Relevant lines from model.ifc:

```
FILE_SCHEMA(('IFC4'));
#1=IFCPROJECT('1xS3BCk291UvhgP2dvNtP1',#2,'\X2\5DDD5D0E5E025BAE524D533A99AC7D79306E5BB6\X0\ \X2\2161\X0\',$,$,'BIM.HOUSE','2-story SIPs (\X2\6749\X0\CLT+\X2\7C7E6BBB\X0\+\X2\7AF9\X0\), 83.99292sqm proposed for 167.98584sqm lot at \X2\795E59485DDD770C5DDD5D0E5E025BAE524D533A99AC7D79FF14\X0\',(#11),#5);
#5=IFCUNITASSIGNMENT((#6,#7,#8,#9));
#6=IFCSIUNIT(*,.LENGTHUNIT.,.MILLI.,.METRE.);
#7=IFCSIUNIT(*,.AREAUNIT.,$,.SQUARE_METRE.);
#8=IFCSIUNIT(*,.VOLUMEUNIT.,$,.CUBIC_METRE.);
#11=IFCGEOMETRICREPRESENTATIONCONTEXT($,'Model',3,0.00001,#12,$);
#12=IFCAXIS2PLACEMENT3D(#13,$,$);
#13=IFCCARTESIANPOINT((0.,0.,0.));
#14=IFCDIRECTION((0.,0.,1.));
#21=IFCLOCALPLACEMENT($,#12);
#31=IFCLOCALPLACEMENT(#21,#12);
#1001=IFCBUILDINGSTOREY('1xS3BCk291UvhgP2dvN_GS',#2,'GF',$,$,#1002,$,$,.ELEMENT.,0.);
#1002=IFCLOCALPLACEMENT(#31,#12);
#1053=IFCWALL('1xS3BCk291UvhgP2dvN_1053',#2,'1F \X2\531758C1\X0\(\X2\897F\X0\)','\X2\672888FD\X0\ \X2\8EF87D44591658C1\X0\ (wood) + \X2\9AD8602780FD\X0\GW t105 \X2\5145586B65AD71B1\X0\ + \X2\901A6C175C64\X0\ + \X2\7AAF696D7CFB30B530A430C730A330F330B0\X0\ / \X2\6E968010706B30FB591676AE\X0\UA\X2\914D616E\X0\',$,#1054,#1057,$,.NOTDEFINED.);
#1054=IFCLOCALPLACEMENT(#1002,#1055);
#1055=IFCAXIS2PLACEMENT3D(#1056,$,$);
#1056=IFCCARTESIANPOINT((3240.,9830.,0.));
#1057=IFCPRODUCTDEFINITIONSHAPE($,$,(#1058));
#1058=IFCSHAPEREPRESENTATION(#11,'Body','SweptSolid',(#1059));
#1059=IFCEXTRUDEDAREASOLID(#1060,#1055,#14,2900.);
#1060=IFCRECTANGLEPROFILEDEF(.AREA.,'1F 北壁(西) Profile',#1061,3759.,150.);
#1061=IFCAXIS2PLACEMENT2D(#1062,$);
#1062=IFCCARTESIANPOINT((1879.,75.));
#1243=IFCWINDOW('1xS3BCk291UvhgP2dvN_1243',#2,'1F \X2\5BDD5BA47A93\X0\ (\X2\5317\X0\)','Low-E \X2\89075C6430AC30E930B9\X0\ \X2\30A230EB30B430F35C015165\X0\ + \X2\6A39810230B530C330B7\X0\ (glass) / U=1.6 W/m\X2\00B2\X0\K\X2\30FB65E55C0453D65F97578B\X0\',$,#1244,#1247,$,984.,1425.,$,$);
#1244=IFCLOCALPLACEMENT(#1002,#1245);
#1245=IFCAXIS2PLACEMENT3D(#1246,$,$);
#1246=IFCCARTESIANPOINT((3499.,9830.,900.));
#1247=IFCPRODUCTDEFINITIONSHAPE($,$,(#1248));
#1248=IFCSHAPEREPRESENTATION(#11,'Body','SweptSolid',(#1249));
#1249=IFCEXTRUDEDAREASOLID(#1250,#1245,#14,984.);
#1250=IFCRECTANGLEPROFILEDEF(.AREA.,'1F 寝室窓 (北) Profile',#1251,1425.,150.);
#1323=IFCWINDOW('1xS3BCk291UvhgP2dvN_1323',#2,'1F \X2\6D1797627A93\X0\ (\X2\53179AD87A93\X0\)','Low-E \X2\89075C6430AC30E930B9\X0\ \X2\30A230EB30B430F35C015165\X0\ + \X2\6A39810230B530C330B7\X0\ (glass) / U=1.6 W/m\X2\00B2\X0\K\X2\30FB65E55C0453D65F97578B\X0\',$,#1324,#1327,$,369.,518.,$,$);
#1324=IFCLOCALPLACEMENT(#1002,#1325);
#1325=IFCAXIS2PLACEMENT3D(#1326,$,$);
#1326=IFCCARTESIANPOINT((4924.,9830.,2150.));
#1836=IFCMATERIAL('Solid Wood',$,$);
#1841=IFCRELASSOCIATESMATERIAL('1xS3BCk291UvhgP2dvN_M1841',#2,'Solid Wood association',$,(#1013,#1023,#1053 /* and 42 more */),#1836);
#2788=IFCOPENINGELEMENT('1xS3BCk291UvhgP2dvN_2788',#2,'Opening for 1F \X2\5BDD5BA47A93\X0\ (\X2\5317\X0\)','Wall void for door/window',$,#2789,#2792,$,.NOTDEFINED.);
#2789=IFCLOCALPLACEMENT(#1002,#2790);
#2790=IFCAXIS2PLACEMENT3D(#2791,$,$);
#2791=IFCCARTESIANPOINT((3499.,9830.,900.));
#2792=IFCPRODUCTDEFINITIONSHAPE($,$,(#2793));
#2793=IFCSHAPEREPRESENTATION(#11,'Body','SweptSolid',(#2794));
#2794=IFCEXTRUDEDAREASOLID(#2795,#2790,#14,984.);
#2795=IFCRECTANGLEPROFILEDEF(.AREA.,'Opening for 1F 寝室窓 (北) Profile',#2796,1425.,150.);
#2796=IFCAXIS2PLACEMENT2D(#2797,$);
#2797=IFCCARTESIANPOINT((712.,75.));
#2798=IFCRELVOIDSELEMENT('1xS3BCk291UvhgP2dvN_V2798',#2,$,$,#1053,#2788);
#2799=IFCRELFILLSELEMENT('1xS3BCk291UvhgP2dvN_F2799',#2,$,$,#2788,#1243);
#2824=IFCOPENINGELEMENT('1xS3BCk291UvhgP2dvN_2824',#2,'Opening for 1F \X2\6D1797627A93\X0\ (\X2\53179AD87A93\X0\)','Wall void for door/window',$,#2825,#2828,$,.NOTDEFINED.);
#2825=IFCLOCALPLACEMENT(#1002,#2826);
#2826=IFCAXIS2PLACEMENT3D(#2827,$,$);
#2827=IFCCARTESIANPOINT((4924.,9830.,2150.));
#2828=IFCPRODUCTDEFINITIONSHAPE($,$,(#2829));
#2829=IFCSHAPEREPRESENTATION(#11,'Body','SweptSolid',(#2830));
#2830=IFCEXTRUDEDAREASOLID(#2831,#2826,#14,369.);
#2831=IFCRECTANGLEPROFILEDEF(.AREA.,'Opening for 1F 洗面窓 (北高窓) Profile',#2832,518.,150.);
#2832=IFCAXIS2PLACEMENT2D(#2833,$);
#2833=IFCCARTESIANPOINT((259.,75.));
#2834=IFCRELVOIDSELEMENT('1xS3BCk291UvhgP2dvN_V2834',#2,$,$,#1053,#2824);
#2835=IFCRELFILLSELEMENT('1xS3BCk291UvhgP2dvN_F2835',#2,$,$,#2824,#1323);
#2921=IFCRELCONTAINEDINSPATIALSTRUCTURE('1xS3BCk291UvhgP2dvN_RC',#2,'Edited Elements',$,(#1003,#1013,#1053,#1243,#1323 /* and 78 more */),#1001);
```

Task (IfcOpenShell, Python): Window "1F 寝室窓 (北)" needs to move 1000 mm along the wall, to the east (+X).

```python
import ifcopenshell
import ifcopenshell.api.geometry
import ifcopenshell.util.placement
import ifcopenshell.util.unit

model = ifcopenshell.open("model.ifc")
unit_scale = ifcopenshell.util.unit.calculate_unit_scale(model)

window = model.by_guid("1xS3BCk291UvhgP2dvN_1243")
opening = window.FillsVoids[0].RelatingOpeningElement
wall = opening.VoidsElements[0].RelatingBuildingElement

wall_matrix = ifcopenshell.util.placement.get_local_placement(wall.ObjectPlacement)
shift = wall_matrix[:3, 0] * 1 / unit_scale
before = ifcopenshell.util.placement.get_local_placement(window.ObjectPlacement)[:3, 3].copy()

# The window is not placed relative to its opening, so move both.
for product in (opening, window):
    matrix = ifcopenshell.util.placement.get_local_placement(product.ObjectPlacement)
    matrix[:3, 3] += shift
    ifcopenshell.api.geometry.edit_object_placement(model, product=product, matrix=matrix, is_si=False)

after = ifcopenshell.util.placement.get_local_placement(window.ObjectPlacement)[:3, 3]
print("window moved by", (after - before).round(3) + 0.0)

model.write("model_updated.ifc")
```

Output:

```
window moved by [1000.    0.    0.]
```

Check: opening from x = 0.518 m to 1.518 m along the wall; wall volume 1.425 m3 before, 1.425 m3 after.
